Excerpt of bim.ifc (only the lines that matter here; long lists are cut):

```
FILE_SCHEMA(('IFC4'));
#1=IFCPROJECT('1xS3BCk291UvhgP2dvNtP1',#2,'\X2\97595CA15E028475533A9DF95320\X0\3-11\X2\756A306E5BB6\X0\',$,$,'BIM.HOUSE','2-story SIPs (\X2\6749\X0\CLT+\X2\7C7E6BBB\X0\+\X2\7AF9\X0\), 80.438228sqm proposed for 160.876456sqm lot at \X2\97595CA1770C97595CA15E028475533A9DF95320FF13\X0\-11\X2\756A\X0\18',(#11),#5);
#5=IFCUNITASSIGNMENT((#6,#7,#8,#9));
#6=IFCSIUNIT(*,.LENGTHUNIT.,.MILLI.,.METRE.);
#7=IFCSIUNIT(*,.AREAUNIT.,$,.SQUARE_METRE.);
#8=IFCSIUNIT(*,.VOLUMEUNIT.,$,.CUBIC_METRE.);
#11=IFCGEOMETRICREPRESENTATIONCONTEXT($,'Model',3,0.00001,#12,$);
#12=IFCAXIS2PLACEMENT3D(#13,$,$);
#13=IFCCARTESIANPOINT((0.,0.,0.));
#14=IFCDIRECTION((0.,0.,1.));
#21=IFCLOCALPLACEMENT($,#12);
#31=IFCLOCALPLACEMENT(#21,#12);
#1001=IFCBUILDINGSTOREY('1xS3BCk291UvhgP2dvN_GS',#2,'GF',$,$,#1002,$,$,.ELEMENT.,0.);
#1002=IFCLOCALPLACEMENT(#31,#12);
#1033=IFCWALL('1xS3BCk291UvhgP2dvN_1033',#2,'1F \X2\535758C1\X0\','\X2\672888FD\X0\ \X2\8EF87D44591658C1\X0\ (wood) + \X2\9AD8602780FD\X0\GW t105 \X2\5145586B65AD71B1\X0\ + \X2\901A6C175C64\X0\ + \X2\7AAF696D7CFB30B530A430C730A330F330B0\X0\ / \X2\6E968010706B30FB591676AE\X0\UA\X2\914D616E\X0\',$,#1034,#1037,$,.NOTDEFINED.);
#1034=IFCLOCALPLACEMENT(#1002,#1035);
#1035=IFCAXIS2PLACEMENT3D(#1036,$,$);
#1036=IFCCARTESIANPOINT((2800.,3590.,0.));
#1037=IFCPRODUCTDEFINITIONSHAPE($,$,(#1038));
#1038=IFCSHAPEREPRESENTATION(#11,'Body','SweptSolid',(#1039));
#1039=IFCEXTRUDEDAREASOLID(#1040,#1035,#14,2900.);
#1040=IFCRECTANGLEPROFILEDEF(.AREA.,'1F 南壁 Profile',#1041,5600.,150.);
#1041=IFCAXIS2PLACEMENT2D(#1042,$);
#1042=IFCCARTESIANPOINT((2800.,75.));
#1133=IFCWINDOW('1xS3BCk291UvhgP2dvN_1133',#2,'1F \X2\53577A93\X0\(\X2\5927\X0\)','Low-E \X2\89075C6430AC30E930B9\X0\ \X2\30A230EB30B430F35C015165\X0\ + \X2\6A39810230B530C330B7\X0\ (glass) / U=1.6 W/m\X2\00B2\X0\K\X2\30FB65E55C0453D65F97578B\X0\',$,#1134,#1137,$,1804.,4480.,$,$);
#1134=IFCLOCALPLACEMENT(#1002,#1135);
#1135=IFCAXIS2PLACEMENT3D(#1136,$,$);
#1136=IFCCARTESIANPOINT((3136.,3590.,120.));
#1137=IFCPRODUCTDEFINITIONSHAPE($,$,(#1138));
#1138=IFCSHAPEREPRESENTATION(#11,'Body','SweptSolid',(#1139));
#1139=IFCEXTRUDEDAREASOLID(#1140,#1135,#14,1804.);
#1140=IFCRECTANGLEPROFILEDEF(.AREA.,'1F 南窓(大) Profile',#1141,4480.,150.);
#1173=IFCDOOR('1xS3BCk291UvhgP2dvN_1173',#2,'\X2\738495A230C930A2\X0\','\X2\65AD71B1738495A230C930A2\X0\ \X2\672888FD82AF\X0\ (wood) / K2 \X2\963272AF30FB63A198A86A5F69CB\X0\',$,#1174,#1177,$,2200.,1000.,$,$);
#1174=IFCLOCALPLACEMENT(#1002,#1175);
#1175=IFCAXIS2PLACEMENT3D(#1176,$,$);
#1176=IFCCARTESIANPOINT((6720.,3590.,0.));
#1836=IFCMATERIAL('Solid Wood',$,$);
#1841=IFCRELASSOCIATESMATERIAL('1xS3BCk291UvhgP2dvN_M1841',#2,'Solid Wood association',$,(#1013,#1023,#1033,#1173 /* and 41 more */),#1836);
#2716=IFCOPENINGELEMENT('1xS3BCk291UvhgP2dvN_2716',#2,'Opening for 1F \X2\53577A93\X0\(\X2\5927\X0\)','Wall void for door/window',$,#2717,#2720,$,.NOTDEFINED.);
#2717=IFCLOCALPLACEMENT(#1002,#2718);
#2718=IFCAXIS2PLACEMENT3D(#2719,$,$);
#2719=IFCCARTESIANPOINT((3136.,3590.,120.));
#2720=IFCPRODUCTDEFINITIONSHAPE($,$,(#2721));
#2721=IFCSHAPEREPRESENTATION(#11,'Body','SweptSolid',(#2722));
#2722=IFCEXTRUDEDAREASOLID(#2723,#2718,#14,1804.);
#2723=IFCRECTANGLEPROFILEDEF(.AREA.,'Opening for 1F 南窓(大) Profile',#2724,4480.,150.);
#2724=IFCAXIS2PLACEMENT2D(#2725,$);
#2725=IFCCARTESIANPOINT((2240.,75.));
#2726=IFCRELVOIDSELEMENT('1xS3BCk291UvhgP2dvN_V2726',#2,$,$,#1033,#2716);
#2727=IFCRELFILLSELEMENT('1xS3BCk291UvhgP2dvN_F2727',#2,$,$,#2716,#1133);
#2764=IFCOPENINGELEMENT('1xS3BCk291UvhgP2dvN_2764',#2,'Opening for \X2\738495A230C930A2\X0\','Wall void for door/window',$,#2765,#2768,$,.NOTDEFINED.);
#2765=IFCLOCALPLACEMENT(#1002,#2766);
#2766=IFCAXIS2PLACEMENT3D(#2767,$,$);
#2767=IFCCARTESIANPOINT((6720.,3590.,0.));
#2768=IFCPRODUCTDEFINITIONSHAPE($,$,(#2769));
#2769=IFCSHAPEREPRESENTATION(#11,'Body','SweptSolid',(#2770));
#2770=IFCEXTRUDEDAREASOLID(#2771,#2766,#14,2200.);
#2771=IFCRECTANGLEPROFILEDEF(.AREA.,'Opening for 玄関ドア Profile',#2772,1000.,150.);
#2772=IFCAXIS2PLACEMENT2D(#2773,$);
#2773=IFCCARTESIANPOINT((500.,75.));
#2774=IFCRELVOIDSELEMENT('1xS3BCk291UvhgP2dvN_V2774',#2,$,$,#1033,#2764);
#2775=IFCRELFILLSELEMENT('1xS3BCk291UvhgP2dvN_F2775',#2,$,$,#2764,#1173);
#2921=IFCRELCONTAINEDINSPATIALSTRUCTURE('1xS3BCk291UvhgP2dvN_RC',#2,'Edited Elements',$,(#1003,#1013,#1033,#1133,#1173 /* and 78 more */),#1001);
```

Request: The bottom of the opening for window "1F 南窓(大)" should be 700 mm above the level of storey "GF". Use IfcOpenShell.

```python
import numpy as np
import ifcopenshell
import ifcopenshell.api.geometry
import ifcopenshell.geom
import ifcopenshell.util.element
import ifcopenshell.util.placement
import ifcopenshell.util.shape
import ifcopenshell.util.unit

model = ifcopenshell.open("bim.ifc")
unit_scale = ifcopenshell.util.unit.calculate_unit_scale(model)

window = model.by_guid("1xS3BCk291UvhgP2dvN_1133")
opening = window.FillsVoids[0].RelatingOpeningElement
storey = ifcopenshell.util.element.get_container(window, ifc_class="IfcBuildingStorey")
level = ifcopenshell.util.placement.get_local_placement(storey.ObjectPlacement)[2, 3]

# The opening's origin need not be at the sill, so measure its lowest point.
shape = ifcopenshell.geom.create_shape(ifcopenshell.geom.settings(), opening)
bottom = ifcopenshell.util.shape.get_shape_bottom_elevation(shape, shape.geometry) / unit_scale
dz = level + 0.7 / unit_scale - bottom

shift = np.array([0.0, 0.0, dz])
# The window is not placed relative to its opening, so move both.
for product in (opening, window):
    matrix = ifcopenshell.util.placement.get_local_placement(product.ObjectPlacement)
    matrix[:3, 3] += shift
    ifcopenshell.api.geometry.edit_object_placement(model, product=product, matrix=matrix, is_si=False)

print(f"moved by {dz * unit_scale:+.3f} m")

model.write("bim_rev.ifc")
```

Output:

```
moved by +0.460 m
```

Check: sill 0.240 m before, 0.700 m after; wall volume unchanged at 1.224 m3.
